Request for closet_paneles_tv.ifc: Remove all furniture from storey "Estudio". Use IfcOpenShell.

First a look at what the model holds.

```python
import ifcopenshell
import ifcopenshell.util.element

model = ifcopenshell.open("closet_paneles_tv.ifc")
print(model.schema)
storey = next(s for s in model.by_type("IfcBuildingStorey") if s.Name == "Estudio")
furniture = [e for e in ifcopenshell.util.element.get_decomposition(storey) if e.is_a("IfcFurnishingElement")]
seen = {}
for e in furniture:
    element_type = ifcopenshell.util.element.get_type(e)
    name = element_type.Name if element_type not in (None, e) else None
    seen[name] = seen.get(name, 0) + 1
for name, count in sorted(seen.items(), key=str):
    print(count, "x", name)
```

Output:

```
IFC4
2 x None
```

```python
import ifcopenshell
import ifcopenshell.api.root
import ifcopenshell.util.element

model = ifcopenshell.open("closet_paneles_tv.ifc")

storey = next(s for s in model.by_type("IfcBuildingStorey") if s.Name == "Estudio")
furniture = [e for e in ifcopenshell.util.element.get_decomposition(storey) if e.is_a("IfcFurnishingElement")]

for e in furniture:
    ifcopenshell.api.root.remove_product(model, product=e)
print(len(furniture), "removed")

model.write("closet_paneles_tv_updated.ifc")
```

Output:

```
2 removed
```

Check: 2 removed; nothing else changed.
